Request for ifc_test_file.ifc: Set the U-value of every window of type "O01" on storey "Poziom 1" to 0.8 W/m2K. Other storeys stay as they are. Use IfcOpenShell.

First a look at what the model holds.

```python
import ifcopenshell
import ifcopenshell.util.element

model = ifcopenshell.open("ifc_test_file.ifc")
print(model.schema)
storey = next(s for s in model.by_type("IfcBuildingStorey") if s.Name == "Poziom 1")
windows = [e for e in ifcopenshell.util.element.get_decomposition(storey) if e.is_a("IfcWindow")]
seen = {}
for e in windows:
    element_type = ifcopenshell.util.element.get_type(e)
    key = (element_type.Name if element_type != e and element_type else None, ifcopenshell.util.element.get_pset(e, "Pset_WindowCommon", "ThermalTransmittance"))
    seen[key] = seen.get(key, 0) + 1
for (name, value), count in sorted(seen.items(), key=str):
    print(count, "x", name, "|", value)
```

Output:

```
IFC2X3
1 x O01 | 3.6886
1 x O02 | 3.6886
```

```python
import ifcopenshell
import ifcopenshell.api.pset
import ifcopenshell.util.element

model = ifcopenshell.open("ifc_test_file.ifc")

storey = next(s for s in model.by_type("IfcBuildingStorey") if s.Name == "Poziom 1")
windows = [e for e in ifcopenshell.util.element.get_decomposition(storey) if e.is_a("IfcWindow")]

count = 0
for e in windows:
    element_type = ifcopenshell.util.element.get_type(e)
    if element_type in (None, e) or element_type.Name != "O01":
        continue
    # add_pset returns the element's existing set when there is one.
    pset = ifcopenshell.api.pset.add_pset(model, product=e, name="Pset_WindowCommon")
    ifcopenshell.api.pset.edit_pset(model, pset=pset, properties={"ThermalTransmittance": 0.8})
    count += 1

print(count, "windows updated")

model.write("ifc_test_file_edited.ifc")
```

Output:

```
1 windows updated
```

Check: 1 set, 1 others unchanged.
